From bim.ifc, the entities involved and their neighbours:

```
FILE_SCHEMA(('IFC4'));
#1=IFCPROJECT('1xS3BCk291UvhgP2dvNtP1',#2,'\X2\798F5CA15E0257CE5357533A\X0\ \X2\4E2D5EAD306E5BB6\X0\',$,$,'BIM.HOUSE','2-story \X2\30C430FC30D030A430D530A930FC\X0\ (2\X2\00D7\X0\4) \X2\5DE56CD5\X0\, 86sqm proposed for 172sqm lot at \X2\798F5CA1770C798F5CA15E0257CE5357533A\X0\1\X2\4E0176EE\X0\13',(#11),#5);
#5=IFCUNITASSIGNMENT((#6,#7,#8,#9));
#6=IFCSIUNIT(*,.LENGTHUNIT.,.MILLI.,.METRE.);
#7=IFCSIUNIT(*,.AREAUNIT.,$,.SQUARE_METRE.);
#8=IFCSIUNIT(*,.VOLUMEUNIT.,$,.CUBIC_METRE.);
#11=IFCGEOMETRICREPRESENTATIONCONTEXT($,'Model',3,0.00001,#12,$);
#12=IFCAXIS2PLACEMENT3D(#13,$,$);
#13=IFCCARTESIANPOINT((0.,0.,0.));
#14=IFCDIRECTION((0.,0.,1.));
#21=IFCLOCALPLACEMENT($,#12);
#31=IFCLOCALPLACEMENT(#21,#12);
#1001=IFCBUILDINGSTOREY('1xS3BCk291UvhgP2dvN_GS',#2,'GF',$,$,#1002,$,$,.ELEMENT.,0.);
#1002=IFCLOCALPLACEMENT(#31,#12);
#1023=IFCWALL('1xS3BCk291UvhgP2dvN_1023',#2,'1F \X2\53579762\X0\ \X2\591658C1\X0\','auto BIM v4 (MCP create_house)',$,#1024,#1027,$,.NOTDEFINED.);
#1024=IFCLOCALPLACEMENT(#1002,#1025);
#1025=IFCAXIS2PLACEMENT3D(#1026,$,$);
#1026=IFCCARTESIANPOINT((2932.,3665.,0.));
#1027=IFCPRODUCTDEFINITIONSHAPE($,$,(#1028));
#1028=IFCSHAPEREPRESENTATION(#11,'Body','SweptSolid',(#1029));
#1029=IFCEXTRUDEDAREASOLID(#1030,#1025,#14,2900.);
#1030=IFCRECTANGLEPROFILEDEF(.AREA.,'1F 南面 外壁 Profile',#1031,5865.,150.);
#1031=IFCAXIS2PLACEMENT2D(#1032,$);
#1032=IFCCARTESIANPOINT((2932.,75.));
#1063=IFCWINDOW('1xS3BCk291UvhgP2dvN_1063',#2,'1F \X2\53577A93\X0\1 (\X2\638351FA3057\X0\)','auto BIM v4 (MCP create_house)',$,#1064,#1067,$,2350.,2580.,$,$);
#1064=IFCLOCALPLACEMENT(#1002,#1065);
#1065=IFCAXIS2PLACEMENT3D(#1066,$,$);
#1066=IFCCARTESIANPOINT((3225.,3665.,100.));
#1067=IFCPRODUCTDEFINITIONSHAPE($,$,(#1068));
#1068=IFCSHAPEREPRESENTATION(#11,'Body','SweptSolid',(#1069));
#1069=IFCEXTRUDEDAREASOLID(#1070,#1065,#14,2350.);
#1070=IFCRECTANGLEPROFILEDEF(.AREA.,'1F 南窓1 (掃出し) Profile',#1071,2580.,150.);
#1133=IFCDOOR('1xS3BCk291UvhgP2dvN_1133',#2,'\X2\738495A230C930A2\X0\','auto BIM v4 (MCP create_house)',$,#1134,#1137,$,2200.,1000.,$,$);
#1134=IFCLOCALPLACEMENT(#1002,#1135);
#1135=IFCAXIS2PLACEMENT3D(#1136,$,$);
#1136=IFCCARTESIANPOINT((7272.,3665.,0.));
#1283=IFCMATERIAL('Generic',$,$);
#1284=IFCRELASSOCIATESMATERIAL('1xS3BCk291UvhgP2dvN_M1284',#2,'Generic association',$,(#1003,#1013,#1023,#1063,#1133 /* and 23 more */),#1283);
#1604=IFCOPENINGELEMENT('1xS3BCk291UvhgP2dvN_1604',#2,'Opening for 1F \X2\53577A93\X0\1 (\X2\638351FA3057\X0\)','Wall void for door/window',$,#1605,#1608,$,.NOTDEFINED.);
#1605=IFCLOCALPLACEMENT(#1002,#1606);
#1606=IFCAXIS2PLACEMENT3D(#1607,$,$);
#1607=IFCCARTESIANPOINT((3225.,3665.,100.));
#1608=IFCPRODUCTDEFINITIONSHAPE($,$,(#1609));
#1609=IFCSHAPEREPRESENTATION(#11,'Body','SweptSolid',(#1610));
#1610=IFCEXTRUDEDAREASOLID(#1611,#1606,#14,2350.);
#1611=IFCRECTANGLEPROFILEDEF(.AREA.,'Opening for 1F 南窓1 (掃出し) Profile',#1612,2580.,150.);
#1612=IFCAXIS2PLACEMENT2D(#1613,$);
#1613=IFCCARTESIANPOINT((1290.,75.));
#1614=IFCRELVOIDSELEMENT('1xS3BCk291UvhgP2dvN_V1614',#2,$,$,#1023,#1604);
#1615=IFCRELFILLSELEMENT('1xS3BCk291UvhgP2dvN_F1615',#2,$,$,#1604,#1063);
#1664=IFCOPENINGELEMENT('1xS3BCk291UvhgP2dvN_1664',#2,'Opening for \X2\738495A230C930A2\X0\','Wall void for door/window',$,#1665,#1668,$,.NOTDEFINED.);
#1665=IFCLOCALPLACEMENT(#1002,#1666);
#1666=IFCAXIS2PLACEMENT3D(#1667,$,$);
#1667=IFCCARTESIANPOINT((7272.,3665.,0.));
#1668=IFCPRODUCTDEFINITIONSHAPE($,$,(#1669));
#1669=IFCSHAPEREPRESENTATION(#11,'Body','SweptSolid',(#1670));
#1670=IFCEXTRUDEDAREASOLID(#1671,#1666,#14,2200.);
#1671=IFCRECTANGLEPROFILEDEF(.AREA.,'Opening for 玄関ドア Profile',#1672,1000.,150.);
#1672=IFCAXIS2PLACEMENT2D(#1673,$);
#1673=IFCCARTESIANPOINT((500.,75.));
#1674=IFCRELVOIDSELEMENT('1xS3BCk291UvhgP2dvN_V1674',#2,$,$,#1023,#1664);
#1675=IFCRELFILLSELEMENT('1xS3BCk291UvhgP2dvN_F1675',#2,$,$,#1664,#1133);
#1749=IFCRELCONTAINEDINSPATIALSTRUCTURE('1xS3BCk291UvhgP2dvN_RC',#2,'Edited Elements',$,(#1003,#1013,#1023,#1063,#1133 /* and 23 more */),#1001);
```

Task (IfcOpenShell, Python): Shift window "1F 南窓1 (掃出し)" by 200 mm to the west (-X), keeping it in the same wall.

```python
import ifcopenshell
import ifcopenshell.api.geometry
import ifcopenshell.util.placement
import ifcopenshell.util.unit

model = ifcopenshell.open("bim.ifc")
unit_scale = ifcopenshell.util.unit.calculate_unit_scale(model)

window = model.by_id(1063)
opening = window.FillsVoids[0].RelatingOpeningElement
wall = opening.VoidsElements[0].RelatingBuildingElement

wall_matrix = ifcopenshell.util.placement.get_local_placement(wall.ObjectPlacement)
shift = wall_matrix[:3, 0] * -0.2 / unit_scale
before = ifcopenshell.util.placement.get_local_placement(window.ObjectPlacement)[:3, 3].copy()

# The window is not placed relative to its opening, so move both.
for product in (opening, window):
    matrix = ifcopenshell.util.placement.get_local_placement(product.ObjectPlacement)
    matrix[:3, 3] += shift
    ifcopenshell.api.geometry.edit_object_placement(model, product=product, matrix=matrix, is_si=False)

after = ifcopenshell.util.placement.get_local_placement(window.ObjectPlacement)[:3, 3]
print("window moved by", (after - before).round(3) + 0.0)

model.write("bim_edited.ifc")
```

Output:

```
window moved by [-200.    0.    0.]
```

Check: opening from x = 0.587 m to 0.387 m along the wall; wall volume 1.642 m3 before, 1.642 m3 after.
